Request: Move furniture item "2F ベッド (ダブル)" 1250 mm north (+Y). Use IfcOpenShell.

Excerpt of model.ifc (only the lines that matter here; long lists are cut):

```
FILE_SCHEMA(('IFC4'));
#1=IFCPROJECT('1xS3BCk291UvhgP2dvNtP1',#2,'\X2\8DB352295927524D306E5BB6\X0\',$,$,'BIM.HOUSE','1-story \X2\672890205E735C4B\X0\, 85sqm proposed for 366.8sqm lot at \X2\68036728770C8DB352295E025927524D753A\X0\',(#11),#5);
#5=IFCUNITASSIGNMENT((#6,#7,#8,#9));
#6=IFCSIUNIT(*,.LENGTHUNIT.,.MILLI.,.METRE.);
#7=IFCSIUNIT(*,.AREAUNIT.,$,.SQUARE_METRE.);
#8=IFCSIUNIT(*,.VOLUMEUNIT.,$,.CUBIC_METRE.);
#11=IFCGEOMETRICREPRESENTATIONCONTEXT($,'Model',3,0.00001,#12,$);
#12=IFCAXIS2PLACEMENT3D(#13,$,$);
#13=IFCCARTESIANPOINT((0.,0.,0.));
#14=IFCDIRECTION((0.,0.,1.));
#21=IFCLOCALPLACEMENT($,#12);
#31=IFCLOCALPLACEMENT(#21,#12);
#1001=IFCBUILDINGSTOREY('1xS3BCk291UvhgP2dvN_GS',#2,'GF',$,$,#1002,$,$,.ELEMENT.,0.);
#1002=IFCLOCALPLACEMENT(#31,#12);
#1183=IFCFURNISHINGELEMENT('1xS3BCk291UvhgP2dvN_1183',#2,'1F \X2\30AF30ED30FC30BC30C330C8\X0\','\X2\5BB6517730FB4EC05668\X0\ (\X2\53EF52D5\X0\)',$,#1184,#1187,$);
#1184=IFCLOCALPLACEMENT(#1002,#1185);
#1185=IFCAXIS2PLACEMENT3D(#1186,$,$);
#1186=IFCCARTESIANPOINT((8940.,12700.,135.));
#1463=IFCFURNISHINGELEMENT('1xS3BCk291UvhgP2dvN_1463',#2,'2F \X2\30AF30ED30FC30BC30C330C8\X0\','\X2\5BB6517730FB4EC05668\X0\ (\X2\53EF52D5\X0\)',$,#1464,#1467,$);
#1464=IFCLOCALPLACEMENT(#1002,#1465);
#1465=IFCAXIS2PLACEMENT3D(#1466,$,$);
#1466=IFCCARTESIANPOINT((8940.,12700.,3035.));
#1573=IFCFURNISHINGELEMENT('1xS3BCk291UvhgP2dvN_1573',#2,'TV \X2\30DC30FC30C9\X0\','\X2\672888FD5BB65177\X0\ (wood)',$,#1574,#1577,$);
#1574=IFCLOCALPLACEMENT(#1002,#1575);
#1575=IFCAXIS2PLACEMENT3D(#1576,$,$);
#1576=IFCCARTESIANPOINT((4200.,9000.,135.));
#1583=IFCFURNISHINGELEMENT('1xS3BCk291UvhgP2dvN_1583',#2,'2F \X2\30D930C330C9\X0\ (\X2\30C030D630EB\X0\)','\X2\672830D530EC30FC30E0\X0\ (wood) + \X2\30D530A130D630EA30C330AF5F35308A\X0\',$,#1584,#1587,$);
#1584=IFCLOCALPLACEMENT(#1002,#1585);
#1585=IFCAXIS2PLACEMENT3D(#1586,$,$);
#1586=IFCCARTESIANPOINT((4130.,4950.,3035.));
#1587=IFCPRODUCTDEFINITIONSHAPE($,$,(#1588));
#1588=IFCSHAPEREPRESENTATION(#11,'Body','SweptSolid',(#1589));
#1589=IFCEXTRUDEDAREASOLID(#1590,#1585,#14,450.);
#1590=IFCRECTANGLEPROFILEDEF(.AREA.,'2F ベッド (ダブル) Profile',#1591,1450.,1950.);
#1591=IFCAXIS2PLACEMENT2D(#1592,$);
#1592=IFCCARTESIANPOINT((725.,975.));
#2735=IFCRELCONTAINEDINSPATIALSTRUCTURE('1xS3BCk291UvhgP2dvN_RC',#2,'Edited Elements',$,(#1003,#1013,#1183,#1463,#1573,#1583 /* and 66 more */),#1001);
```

```python
import ifcopenshell
import ifcopenshell.api.geometry
import ifcopenshell.util.placement

model = ifcopenshell.open("model.ifc")

item = model.by_guid("1xS3BCk291UvhgP2dvN_1583")
matrix = ifcopenshell.util.placement.get_local_placement(item.ObjectPlacement)
matrix[1, 3] += 1250.0
ifcopenshell.api.geometry.edit_object_placement(model, product=item, matrix=matrix, is_si=False)

print(ifcopenshell.util.placement.get_local_placement(item.ObjectPlacement).round(3) + 0.0)

model.write("model_updated.ifc")
```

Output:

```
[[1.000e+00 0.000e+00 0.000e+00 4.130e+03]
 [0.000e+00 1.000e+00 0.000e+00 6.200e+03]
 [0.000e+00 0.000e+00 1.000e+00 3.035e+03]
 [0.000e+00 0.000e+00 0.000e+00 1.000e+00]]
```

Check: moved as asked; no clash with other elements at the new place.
